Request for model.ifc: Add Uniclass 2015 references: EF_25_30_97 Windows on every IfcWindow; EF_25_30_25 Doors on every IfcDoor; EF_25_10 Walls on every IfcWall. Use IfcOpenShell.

First a look at what the model holds.

```python
import ifcopenshell

model = ifcopenshell.open("model.ifc")
print(model.schema)
print("classifications:", [c.Name for c in model.by_type("IfcClassification")])
for ifc_class in ("IfcDoor", "IfcRoof", "IfcStair", "IfcWall", "IfcWindow"):
    print(ifc_class, len(model.by_type(ifc_class)))
```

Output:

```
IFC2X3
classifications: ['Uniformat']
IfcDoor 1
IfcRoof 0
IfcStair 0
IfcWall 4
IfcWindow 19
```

```python
import ifcopenshell
import ifcopenshell.api.classification

model = ifcopenshell.open("model.ifc")

# IFC2X3 requires Source and Edition and has no link from the project to the system.
system = model.create_entity("IfcClassification", Source="NBS", Edition="2015", Name="Uniclass 2015")

codes = {
    "IfcWindow": ("EF_25_30_97", "Windows"),
    "IfcDoor": ("EF_25_30_25", "Doors"),
    "IfcWall": ("EF_25_10", "Walls"),
}
for ifc_class, (code, name) in codes.items():
    products = model.by_type(ifc_class)
    ifcopenshell.api.classification.add_reference(
        model, products=products, classification=system, identification=code, name=name
    )
    print(code, len(products))

model.write("model-out.ifc")
```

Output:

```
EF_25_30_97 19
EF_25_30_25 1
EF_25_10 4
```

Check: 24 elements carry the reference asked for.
